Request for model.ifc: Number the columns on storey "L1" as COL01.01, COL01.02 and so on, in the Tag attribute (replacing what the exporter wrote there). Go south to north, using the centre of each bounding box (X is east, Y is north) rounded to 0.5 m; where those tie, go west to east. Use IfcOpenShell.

First a look at what the model holds.

```python
import ifcopenshell
import ifcopenshell.util.element
import ifcopenshell.util.placement

model = ifcopenshell.open("model.ifc")
print(model.schema)
storey = next(s for s in model.by_type("IfcBuildingStorey") if s.Name == "L1")
columns = [e for e in ifcopenshell.util.element.get_decomposition(storey) if e.is_a("IfcColumn")]
for e in sorted(columns, key=lambda e: e.id()):
    origin = ifcopenshell.util.placement.get_local_placement(e.ObjectPlacement)[:3, 3]
    print(e.id(), e.Tag, e.Name, origin.round(2) + 0.0, sep=" | ")
```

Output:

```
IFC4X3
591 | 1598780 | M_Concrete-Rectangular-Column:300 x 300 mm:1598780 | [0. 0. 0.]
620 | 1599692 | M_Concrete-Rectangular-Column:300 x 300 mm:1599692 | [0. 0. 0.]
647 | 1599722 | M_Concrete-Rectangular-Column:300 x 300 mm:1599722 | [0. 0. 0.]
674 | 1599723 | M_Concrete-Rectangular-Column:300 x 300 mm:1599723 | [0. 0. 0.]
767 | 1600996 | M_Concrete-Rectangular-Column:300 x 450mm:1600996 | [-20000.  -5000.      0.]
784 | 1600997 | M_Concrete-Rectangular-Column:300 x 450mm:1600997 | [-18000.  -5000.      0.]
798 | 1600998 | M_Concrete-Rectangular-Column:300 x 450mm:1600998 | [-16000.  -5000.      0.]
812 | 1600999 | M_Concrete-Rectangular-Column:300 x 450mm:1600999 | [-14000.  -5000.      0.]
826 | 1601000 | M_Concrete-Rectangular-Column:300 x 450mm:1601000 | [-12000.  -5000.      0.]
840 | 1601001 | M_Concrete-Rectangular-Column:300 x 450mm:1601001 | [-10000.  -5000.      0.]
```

```python
import ifcopenshell
import ifcopenshell.geom
import ifcopenshell.util.element
import ifcopenshell.util.shape

model = ifcopenshell.open("model.ifc")
settings = ifcopenshell.geom.settings()
settings.set("use-world-coords", True)


def centre(element):
    shape = ifcopenshell.geom.create_shape(settings, element)
    return ifcopenshell.util.shape.get_bbox_centroid(shape.geometry)


storey = next(s for s in model.by_type("IfcBuildingStorey") if s.Name == "L1")
columns = [e for e in ifcopenshell.util.element.get_decomposition(storey) if e.is_a("IfcColumn")]

# Insertion points can sit at a corner or the storey origin, so sort by the geometry (in metres).
centres = {e: centre(e) for e in columns}
columns.sort(key=lambda e: (round(centres[e][1] / 0.5), centres[e][0]))

for i, e in enumerate(columns, start=1):
    number = f"COL01.{i:02d}"
    e.Tag = number
    print(e.id(), number)

model.write("model_rev.ifc")
```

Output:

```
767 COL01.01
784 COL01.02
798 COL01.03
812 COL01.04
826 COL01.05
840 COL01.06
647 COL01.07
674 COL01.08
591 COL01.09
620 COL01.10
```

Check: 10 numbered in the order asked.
